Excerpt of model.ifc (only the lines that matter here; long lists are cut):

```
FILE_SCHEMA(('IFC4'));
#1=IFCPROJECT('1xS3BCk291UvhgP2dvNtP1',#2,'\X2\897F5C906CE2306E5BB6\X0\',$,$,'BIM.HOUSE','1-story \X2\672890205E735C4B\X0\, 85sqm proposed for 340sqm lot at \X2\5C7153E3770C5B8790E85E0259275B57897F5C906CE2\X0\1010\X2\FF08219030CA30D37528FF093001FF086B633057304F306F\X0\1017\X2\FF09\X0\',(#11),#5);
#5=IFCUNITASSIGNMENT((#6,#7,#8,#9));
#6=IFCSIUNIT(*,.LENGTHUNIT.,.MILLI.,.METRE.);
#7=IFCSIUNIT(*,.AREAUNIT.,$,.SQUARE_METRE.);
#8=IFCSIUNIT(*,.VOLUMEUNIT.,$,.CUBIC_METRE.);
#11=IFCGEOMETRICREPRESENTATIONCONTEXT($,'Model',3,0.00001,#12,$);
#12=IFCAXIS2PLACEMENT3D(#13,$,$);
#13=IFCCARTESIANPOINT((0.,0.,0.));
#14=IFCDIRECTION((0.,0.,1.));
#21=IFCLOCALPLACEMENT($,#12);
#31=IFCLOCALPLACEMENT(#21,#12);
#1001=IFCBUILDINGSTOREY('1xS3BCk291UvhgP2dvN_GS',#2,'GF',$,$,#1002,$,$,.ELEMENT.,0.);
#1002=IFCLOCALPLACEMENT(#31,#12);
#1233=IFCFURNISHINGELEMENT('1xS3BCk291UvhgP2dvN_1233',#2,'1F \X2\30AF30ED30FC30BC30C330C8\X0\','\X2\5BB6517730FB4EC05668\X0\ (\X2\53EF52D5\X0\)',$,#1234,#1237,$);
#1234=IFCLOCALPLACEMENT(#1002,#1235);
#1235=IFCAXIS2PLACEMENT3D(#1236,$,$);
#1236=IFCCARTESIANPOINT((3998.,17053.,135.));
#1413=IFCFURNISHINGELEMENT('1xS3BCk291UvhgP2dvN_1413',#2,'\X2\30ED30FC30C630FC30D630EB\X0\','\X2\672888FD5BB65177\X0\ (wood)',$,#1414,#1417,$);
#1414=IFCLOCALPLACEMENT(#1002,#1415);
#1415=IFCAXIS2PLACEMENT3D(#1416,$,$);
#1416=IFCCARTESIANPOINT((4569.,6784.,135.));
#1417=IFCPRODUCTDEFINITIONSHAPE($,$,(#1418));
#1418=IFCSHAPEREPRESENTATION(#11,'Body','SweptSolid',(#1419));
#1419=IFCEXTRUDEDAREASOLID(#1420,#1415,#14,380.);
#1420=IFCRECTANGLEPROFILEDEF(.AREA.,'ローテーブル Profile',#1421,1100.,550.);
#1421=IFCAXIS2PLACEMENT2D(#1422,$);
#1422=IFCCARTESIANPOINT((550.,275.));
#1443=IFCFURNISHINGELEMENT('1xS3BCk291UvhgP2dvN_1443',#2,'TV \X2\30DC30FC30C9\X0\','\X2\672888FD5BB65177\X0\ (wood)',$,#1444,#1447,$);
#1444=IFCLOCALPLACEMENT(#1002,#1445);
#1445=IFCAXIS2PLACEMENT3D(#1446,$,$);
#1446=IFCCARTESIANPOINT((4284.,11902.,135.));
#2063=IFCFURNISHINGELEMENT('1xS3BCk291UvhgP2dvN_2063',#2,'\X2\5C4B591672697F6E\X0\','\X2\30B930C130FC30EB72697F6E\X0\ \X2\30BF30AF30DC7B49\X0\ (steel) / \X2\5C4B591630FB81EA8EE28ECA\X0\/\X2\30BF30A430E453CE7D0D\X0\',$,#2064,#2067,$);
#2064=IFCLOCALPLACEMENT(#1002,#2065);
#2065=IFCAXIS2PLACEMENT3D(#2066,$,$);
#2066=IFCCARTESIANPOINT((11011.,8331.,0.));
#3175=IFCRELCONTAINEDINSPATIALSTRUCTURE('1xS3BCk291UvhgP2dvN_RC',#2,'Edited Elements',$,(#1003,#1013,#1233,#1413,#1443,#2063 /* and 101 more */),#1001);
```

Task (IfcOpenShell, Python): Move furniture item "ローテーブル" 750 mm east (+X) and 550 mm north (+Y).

```python
import ifcopenshell
import ifcopenshell.api.geometry
import ifcopenshell.util.placement
import ifcopenshell.util.unit

model = ifcopenshell.open("model.ifc")
unit_scale = ifcopenshell.util.unit.calculate_unit_scale(model)

item = model.by_guid("1xS3BCk291UvhgP2dvN_1413")
matrix = ifcopenshell.util.placement.get_local_placement(item.ObjectPlacement)
matrix[0, 3] += 0.75 / unit_scale
matrix[1, 3] += 0.55 / unit_scale
ifcopenshell.api.geometry.edit_object_placement(model, product=item, matrix=matrix, is_si=False)

print(ifcopenshell.util.placement.get_local_placement(item.ObjectPlacement).round(3) + 0.0)

model.write("model_edited.ifc")
```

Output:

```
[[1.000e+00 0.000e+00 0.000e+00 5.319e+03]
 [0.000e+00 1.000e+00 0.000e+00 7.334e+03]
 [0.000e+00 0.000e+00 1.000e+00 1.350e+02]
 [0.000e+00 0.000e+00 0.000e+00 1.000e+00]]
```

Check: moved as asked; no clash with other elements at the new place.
